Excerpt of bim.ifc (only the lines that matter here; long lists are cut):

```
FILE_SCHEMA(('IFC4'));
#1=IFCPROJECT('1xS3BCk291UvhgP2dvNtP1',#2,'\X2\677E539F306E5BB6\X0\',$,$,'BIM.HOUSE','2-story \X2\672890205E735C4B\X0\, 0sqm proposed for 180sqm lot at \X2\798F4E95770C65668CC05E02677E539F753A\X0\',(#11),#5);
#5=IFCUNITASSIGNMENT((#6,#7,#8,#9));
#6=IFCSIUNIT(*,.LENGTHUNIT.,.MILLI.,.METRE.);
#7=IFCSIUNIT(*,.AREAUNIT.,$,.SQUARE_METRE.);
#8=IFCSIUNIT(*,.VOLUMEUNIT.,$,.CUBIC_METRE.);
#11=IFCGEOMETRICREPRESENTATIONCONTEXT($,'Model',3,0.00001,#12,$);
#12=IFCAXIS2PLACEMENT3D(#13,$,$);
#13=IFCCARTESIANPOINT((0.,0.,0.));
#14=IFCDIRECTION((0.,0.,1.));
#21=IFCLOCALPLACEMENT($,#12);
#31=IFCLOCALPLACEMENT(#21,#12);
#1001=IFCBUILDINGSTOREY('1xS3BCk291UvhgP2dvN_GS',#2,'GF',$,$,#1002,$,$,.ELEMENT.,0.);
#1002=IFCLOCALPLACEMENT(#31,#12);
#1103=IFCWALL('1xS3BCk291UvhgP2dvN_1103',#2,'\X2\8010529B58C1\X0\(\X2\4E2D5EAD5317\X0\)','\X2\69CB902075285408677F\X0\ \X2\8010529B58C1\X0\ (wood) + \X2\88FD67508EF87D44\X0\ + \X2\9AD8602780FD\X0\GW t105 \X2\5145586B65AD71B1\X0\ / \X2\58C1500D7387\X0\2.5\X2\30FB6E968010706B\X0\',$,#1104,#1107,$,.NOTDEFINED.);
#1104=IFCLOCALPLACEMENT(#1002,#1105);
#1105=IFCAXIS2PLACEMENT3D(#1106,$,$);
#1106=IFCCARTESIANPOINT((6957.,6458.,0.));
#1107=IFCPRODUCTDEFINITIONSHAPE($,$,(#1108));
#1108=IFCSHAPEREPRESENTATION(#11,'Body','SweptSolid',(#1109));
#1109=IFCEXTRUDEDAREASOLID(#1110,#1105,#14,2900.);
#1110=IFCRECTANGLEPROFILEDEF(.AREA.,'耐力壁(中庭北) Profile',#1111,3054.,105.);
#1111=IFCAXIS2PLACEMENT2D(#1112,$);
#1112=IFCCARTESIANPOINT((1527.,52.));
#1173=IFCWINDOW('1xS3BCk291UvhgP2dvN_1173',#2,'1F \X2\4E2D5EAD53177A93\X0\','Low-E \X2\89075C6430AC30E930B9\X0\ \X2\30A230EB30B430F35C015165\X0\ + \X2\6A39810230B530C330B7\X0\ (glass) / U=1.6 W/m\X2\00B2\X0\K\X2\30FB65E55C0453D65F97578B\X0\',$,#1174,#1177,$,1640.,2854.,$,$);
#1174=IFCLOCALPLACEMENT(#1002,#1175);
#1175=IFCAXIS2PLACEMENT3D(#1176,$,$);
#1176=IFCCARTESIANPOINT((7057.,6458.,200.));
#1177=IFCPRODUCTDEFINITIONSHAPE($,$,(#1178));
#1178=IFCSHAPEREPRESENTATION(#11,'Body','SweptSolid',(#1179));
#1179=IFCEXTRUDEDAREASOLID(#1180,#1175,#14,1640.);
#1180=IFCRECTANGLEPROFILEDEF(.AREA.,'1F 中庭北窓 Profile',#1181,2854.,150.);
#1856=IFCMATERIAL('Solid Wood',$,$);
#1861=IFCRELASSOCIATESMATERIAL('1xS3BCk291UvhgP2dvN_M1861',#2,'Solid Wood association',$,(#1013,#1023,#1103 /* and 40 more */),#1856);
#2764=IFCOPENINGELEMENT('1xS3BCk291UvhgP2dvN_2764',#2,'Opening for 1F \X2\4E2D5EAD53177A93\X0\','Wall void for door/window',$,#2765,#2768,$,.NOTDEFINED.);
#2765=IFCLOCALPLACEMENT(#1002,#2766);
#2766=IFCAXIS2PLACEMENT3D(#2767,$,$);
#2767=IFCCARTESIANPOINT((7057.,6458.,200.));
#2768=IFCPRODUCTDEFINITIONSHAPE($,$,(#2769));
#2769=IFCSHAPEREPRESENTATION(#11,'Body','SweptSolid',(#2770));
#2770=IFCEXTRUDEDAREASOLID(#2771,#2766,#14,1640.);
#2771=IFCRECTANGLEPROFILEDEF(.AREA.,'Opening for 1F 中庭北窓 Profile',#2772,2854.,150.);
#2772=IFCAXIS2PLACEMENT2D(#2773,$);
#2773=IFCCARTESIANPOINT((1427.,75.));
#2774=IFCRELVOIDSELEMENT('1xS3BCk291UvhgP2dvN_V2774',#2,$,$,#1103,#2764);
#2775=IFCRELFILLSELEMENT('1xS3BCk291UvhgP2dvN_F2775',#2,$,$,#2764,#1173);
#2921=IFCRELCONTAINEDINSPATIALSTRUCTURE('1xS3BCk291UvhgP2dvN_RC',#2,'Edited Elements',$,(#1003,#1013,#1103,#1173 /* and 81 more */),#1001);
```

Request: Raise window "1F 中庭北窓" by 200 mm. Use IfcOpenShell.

```python
import numpy as np
import ifcopenshell
import ifcopenshell.api.geometry
import ifcopenshell.util.placement
import ifcopenshell.util.unit

model = ifcopenshell.open("bim.ifc")
unit_scale = ifcopenshell.util.unit.calculate_unit_scale(model)

window = model.by_guid("1xS3BCk291UvhgP2dvN_1173")
opening = window.FillsVoids[0].RelatingOpeningElement
dz = 0.2 / unit_scale

shift = np.array([0.0, 0.0, dz])
# The window is not placed relative to its opening, so move both.
for product in (opening, window):
    matrix = ifcopenshell.util.placement.get_local_placement(product.ObjectPlacement)
    matrix[:3, 3] += shift
    ifcopenshell.api.geometry.edit_object_placement(model, product=product, matrix=matrix, is_si=False)

print(f"moved by {dz * unit_scale:+.3f} m")

model.write("bim_rev.ifc")
```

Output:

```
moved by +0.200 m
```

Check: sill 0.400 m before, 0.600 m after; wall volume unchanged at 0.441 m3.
